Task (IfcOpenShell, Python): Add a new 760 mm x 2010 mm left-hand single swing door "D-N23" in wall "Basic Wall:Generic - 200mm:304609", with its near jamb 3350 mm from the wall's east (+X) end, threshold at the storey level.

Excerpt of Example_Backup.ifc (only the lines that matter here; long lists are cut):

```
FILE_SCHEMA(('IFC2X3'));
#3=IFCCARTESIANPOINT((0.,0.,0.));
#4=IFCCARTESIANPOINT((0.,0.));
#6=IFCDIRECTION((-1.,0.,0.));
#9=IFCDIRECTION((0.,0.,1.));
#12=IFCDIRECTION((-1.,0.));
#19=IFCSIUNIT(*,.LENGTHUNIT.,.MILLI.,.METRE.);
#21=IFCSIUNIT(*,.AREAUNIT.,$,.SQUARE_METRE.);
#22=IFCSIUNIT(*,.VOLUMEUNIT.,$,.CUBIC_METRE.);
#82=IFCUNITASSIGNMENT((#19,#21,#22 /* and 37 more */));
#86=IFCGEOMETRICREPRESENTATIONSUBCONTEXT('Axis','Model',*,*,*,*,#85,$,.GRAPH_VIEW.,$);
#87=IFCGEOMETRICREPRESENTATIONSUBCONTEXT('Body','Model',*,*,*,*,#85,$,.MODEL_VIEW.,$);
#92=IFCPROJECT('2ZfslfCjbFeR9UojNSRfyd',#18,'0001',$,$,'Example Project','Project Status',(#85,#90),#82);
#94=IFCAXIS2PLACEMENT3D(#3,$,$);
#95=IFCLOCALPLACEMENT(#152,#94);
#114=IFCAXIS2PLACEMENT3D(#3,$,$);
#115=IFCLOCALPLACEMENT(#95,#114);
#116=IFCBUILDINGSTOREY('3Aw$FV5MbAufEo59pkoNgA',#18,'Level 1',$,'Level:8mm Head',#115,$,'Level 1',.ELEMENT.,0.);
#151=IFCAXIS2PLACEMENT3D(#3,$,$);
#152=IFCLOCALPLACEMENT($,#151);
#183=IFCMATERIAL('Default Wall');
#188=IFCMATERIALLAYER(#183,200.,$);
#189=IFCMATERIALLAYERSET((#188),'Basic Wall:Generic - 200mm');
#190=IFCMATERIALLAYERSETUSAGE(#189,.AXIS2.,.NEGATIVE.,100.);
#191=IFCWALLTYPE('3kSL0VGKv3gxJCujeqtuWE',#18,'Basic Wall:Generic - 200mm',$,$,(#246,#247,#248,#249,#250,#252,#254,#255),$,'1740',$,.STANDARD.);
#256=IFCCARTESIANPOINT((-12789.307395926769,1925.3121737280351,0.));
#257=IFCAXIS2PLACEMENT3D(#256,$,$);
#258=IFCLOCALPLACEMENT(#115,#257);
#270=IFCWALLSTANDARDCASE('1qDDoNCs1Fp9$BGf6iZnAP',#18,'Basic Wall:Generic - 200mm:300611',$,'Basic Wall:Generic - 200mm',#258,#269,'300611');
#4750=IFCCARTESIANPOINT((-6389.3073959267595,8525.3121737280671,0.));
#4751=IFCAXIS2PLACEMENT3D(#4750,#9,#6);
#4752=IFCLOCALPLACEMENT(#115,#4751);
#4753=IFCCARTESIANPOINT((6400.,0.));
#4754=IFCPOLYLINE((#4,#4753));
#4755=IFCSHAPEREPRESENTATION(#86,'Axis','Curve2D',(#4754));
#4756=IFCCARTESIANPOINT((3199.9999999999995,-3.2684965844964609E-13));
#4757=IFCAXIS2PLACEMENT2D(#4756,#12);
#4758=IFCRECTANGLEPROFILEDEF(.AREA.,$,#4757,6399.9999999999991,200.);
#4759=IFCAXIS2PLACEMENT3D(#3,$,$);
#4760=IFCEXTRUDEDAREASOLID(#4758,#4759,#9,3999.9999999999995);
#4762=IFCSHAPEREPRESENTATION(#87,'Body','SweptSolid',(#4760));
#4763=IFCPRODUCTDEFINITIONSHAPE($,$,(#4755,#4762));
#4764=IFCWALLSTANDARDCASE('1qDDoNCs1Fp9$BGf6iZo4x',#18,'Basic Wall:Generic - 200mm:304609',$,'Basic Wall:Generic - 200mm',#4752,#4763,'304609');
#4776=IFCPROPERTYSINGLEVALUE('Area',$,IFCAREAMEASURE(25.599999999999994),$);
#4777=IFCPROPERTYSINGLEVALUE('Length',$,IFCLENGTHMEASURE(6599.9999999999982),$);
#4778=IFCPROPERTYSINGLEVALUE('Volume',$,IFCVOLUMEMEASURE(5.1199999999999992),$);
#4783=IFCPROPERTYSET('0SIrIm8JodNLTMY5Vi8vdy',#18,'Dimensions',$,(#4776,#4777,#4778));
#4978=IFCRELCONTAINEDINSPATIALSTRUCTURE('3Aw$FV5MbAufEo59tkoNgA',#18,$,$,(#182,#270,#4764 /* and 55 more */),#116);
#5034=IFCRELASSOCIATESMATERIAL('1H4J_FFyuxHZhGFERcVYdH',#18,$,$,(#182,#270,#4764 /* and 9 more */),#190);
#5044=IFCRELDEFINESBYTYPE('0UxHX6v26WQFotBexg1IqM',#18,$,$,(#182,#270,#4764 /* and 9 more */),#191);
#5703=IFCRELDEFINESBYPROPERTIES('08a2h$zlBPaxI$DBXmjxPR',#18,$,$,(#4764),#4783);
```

```python
import numpy as np
import ifcopenshell
import ifcopenshell.api.feature
import ifcopenshell.api.geometry
import ifcopenshell.api.pset
import ifcopenshell.api.root
import ifcopenshell.api.spatial
import ifcopenshell.api.type
import ifcopenshell.geom
import ifcopenshell.util.element
import ifcopenshell.util.placement
import ifcopenshell.util.representation
import ifcopenshell.util.shape
import ifcopenshell.util.unit

model = ifcopenshell.open("Example_Backup.ifc")
unit_scale = ifcopenshell.util.unit.calculate_unit_scale(model)
area_scale = ifcopenshell.util.unit.calculate_unit_scale(model, "AREAUNIT")
volume_scale = ifcopenshell.util.unit.calculate_unit_scale(model, "VOLUMEUNIT")
settings = ifcopenshell.geom.settings()


def volume(element):
    """Net volume in cubic metres, openings subtracted."""
    shape = ifcopenshell.geom.create_shape(settings, element)
    return ifcopenshell.util.shape.get_volume(shape.geometry)


wall = model.by_guid("1qDDoNCs1Fp9$BGf6iZo4x")
storey = ifcopenshell.util.element.get_container(wall, ifc_class="IfcBuildingStorey")
context = ifcopenshell.util.representation.get_context(model, "Model", "Body", "MODEL_VIEW")
before = volume(wall)

width, height, from_end, sill = 0.76, 2.01, 3.35, 0.0  # metres

# The wall runs along its own X axis, and the end named is its -X end.
wall_shape = ifcopenshell.geom.create_shape(settings, wall)
x, y, z = ifcopenshell.util.shape.get_vertices(wall_shape.geometry).T
start = x.min() + from_end
face, thickness = float(y.min()), float(y.max() - y.min())
wall_matrix = ifcopenshell.util.placement.get_local_placement(wall.ObjectPlacement)
level = ifcopenshell.util.placement.get_local_placement(storey.ObjectPlacement)[2, 3]


def in_wall(x, y):
    """Placement at x, y metres in the wall's axes, at sill height."""
    matrix = wall_matrix.copy()
    matrix[:, 3] = wall_matrix @ np.array([x / unit_scale, y / unit_scale, 0.0, 1.0])
    matrix[2, 3] = level + sill / unit_scale
    return matrix


# Opening: a box that overshoots both wall faces by 50 mm.
opening = ifcopenshell.api.root.create_entity(model, ifc_class="IfcOpeningElement")
box = ifcopenshell.api.geometry.add_wall_representation(
    model, context=context, length=width, height=height, thickness=thickness + 0.1
)
ifcopenshell.api.geometry.assign_representation(model, product=opening, representation=box)
ifcopenshell.api.geometry.edit_object_placement(model, product=opening, matrix=in_wall(start, face - 0.05), is_si=False)
ifcopenshell.api.feature.add_feature(model, feature=opening, element=wall)

door = ifcopenshell.api.root.create_entity(model, ifc_class="IfcDoor", name="D-N23")
door.OverallWidth, door.OverallHeight = width / unit_scale, height / unit_scale
body = ifcopenshell.api.geometry.add_door_representation(
    model,
    context=context,
    overall_width=door.OverallWidth,
    overall_height=door.OverallHeight,
    operation_type="SINGLE_SWING_LEFT",
    lining_properties={"LiningDepth": thickness / unit_scale, "ThresholdDepth": thickness / unit_scale},
)
ifcopenshell.api.geometry.assign_representation(model, product=door, representation=body)
ifcopenshell.api.spatial.assign_container(model, products=[door], relating_structure=storey)
fills = ifcopenshell.api.feature.add_filling(model, opening=opening, element=door)
fills.OwnerHistory = door.OwnerHistory  # required in IFC2X3

# IFC2X3 keeps the operation on the door style.
style = ifcopenshell.api.root.create_entity(model, ifc_class="IfcDoorStyle", name="D-N23")
style.OperationType, style.ConstructionType = "SINGLE_SWING_LEFT", "NOTDEFINED"
style.ParameterTakesPrecedence = style.Sizeable = False
ifcopenshell.api.type.assign_type(model, related_objects=[door], relating_type=style)

# The lining spans the wall, so the door starts at the wall face.
ifcopenshell.api.geometry.edit_object_placement(model, product=door, matrix=in_wall(start, face), is_si=False)

after = volume(wall)

# Update the wall's stored quantities.
pset = model.by_id(ifcopenshell.util.element.get_pset(wall, "Dimensions", should_inherit=False)["id"])
ifcopenshell.api.pset.edit_pset(model, pset=pset, properties={
    "Area": model.create_entity("IfcAreaMeasure", after / thickness / area_scale),
    "Volume": model.create_entity("IfcVolumeMeasure", after / volume_scale),
})

print(f"wall volume {before:.3f} -> {after:.3f} m3")

model.write("Example_Backup_rev.ifc")
```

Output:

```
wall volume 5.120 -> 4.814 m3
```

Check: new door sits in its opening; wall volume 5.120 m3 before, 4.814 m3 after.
